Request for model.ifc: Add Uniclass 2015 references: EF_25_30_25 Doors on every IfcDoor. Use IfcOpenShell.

First a look at what the model holds.

```python
import ifcopenshell

model = ifcopenshell.open("model.ifc")
print(model.schema)
print("classifications:", [c.Name for c in model.by_type("IfcClassification")])
for ifc_class in ("IfcDoor", "IfcRoof", "IfcStair", "IfcWall", "IfcWindow"):
    print(ifc_class, len(model.by_type(ifc_class)))
```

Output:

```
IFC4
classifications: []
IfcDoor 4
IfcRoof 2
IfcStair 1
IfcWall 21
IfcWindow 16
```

```python
import ifcopenshell
import ifcopenshell.api.classification

model = ifcopenshell.open("model.ifc")

system = ifcopenshell.api.classification.add_classification(model, classification="Uniclass 2015")

codes = {
    "IfcDoor": ("EF_25_30_25", "Doors"),
}
for ifc_class, (code, name) in codes.items():
    products = model.by_type(ifc_class)
    ifcopenshell.api.classification.add_reference(
        model, products=products, classification=system, identification=code, name=name
    )
    print(code, len(products))

model.write("model_rev.ifc")
```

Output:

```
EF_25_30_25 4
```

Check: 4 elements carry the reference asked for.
